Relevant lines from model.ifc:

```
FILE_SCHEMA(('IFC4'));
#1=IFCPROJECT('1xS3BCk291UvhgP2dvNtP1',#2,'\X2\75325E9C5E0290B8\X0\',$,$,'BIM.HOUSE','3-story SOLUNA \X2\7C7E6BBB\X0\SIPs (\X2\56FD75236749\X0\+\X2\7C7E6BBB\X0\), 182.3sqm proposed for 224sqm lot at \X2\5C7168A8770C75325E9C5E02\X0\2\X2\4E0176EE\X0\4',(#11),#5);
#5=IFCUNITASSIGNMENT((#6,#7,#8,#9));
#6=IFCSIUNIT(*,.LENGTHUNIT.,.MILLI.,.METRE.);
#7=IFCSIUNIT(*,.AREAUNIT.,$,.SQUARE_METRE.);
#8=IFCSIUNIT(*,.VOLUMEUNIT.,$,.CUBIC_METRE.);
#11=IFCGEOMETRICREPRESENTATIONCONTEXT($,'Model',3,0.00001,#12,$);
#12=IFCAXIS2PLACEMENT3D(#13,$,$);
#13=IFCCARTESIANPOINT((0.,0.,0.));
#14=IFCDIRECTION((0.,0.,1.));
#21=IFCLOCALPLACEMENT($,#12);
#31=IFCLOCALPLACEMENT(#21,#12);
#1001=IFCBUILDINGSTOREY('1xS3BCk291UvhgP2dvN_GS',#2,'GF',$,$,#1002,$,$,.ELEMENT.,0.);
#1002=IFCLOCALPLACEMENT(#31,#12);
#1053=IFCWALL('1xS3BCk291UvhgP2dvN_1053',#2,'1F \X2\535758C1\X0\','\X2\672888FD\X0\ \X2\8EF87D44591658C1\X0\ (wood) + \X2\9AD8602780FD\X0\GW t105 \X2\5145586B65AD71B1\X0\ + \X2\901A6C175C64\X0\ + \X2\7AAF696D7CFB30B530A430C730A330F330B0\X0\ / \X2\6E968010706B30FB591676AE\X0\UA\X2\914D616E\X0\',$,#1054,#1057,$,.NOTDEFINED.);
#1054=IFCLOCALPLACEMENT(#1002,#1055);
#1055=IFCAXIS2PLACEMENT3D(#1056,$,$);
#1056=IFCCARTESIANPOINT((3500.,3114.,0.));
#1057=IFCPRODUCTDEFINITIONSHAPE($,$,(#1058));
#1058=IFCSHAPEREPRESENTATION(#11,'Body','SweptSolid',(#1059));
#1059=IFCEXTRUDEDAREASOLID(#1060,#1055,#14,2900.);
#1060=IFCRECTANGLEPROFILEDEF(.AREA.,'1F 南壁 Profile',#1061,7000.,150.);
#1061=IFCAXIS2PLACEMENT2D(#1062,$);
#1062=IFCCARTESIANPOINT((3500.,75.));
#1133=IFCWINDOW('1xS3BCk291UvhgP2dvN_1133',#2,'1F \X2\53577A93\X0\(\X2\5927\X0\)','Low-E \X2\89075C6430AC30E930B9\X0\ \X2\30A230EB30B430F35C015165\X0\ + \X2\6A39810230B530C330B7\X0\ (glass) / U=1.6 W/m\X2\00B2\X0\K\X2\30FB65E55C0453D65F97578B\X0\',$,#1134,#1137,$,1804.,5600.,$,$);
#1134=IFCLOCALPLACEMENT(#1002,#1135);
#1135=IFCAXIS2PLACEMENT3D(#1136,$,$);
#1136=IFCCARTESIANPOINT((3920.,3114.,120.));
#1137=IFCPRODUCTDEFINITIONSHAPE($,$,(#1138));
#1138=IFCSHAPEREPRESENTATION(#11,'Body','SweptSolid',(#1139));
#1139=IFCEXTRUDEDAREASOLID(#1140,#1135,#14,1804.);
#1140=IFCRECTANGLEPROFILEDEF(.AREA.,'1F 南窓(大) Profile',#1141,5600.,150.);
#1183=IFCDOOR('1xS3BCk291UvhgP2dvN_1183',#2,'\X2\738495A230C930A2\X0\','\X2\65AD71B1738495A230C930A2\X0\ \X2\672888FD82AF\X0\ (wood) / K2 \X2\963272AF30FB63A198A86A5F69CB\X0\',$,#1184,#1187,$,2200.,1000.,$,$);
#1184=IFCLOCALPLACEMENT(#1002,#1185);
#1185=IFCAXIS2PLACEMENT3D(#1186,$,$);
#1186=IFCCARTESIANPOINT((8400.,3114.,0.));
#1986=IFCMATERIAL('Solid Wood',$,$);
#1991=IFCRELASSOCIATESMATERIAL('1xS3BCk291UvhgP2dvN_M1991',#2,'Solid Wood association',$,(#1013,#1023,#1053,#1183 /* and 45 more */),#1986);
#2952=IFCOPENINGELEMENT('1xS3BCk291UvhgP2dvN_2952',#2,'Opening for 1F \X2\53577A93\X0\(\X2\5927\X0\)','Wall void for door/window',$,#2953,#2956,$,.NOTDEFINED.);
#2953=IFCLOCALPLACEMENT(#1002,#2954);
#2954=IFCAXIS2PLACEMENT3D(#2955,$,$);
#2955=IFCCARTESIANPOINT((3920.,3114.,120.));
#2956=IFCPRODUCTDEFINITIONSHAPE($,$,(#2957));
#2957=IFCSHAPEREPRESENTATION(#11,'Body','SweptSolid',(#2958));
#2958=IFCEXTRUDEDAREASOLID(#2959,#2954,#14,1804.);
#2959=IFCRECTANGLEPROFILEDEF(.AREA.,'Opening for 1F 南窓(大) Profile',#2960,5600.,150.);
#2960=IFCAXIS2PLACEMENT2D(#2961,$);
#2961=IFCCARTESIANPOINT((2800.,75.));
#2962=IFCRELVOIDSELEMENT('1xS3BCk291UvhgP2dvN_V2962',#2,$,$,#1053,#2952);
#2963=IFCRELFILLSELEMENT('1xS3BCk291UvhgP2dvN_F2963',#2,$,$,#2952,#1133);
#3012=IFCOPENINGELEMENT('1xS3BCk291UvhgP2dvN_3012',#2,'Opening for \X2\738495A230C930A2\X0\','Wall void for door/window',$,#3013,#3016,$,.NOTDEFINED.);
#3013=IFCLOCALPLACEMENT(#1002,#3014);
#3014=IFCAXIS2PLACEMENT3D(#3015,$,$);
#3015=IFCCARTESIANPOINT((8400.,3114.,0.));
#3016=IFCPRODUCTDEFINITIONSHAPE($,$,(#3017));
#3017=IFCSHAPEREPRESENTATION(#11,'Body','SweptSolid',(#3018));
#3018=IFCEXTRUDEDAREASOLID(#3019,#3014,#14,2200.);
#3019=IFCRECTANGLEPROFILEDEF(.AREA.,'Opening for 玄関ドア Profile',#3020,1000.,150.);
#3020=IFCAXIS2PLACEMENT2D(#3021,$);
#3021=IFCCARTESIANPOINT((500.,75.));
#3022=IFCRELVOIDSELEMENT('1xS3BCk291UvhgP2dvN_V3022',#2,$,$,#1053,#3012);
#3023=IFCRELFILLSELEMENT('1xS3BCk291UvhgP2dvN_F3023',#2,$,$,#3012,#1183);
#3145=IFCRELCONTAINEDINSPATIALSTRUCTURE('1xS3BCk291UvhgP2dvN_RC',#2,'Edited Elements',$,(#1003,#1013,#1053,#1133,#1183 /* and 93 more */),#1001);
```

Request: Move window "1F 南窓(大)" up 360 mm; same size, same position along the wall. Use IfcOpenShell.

```python
import numpy as np
import ifcopenshell
import ifcopenshell.api.geometry
import ifcopenshell.util.placement
import ifcopenshell.util.unit

model = ifcopenshell.open("model.ifc")
unit_scale = ifcopenshell.util.unit.calculate_unit_scale(model)

window = model.by_id(1133)
opening = window.FillsVoids[0].RelatingOpeningElement
dz = 360.0

shift = np.array([0.0, 0.0, dz])
# The window is not placed relative to its opening, so move both.
for product in (opening, window):
    matrix = ifcopenshell.util.placement.get_local_placement(product.ObjectPlacement)
    matrix[:3, 3] += shift
    ifcopenshell.api.geometry.edit_object_placement(model, product=product, matrix=matrix, is_si=False)

print(f"moved by {dz * unit_scale:+.3f} m")

model.write("model-out.ifc")
```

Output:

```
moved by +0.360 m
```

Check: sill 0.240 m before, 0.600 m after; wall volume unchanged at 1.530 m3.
